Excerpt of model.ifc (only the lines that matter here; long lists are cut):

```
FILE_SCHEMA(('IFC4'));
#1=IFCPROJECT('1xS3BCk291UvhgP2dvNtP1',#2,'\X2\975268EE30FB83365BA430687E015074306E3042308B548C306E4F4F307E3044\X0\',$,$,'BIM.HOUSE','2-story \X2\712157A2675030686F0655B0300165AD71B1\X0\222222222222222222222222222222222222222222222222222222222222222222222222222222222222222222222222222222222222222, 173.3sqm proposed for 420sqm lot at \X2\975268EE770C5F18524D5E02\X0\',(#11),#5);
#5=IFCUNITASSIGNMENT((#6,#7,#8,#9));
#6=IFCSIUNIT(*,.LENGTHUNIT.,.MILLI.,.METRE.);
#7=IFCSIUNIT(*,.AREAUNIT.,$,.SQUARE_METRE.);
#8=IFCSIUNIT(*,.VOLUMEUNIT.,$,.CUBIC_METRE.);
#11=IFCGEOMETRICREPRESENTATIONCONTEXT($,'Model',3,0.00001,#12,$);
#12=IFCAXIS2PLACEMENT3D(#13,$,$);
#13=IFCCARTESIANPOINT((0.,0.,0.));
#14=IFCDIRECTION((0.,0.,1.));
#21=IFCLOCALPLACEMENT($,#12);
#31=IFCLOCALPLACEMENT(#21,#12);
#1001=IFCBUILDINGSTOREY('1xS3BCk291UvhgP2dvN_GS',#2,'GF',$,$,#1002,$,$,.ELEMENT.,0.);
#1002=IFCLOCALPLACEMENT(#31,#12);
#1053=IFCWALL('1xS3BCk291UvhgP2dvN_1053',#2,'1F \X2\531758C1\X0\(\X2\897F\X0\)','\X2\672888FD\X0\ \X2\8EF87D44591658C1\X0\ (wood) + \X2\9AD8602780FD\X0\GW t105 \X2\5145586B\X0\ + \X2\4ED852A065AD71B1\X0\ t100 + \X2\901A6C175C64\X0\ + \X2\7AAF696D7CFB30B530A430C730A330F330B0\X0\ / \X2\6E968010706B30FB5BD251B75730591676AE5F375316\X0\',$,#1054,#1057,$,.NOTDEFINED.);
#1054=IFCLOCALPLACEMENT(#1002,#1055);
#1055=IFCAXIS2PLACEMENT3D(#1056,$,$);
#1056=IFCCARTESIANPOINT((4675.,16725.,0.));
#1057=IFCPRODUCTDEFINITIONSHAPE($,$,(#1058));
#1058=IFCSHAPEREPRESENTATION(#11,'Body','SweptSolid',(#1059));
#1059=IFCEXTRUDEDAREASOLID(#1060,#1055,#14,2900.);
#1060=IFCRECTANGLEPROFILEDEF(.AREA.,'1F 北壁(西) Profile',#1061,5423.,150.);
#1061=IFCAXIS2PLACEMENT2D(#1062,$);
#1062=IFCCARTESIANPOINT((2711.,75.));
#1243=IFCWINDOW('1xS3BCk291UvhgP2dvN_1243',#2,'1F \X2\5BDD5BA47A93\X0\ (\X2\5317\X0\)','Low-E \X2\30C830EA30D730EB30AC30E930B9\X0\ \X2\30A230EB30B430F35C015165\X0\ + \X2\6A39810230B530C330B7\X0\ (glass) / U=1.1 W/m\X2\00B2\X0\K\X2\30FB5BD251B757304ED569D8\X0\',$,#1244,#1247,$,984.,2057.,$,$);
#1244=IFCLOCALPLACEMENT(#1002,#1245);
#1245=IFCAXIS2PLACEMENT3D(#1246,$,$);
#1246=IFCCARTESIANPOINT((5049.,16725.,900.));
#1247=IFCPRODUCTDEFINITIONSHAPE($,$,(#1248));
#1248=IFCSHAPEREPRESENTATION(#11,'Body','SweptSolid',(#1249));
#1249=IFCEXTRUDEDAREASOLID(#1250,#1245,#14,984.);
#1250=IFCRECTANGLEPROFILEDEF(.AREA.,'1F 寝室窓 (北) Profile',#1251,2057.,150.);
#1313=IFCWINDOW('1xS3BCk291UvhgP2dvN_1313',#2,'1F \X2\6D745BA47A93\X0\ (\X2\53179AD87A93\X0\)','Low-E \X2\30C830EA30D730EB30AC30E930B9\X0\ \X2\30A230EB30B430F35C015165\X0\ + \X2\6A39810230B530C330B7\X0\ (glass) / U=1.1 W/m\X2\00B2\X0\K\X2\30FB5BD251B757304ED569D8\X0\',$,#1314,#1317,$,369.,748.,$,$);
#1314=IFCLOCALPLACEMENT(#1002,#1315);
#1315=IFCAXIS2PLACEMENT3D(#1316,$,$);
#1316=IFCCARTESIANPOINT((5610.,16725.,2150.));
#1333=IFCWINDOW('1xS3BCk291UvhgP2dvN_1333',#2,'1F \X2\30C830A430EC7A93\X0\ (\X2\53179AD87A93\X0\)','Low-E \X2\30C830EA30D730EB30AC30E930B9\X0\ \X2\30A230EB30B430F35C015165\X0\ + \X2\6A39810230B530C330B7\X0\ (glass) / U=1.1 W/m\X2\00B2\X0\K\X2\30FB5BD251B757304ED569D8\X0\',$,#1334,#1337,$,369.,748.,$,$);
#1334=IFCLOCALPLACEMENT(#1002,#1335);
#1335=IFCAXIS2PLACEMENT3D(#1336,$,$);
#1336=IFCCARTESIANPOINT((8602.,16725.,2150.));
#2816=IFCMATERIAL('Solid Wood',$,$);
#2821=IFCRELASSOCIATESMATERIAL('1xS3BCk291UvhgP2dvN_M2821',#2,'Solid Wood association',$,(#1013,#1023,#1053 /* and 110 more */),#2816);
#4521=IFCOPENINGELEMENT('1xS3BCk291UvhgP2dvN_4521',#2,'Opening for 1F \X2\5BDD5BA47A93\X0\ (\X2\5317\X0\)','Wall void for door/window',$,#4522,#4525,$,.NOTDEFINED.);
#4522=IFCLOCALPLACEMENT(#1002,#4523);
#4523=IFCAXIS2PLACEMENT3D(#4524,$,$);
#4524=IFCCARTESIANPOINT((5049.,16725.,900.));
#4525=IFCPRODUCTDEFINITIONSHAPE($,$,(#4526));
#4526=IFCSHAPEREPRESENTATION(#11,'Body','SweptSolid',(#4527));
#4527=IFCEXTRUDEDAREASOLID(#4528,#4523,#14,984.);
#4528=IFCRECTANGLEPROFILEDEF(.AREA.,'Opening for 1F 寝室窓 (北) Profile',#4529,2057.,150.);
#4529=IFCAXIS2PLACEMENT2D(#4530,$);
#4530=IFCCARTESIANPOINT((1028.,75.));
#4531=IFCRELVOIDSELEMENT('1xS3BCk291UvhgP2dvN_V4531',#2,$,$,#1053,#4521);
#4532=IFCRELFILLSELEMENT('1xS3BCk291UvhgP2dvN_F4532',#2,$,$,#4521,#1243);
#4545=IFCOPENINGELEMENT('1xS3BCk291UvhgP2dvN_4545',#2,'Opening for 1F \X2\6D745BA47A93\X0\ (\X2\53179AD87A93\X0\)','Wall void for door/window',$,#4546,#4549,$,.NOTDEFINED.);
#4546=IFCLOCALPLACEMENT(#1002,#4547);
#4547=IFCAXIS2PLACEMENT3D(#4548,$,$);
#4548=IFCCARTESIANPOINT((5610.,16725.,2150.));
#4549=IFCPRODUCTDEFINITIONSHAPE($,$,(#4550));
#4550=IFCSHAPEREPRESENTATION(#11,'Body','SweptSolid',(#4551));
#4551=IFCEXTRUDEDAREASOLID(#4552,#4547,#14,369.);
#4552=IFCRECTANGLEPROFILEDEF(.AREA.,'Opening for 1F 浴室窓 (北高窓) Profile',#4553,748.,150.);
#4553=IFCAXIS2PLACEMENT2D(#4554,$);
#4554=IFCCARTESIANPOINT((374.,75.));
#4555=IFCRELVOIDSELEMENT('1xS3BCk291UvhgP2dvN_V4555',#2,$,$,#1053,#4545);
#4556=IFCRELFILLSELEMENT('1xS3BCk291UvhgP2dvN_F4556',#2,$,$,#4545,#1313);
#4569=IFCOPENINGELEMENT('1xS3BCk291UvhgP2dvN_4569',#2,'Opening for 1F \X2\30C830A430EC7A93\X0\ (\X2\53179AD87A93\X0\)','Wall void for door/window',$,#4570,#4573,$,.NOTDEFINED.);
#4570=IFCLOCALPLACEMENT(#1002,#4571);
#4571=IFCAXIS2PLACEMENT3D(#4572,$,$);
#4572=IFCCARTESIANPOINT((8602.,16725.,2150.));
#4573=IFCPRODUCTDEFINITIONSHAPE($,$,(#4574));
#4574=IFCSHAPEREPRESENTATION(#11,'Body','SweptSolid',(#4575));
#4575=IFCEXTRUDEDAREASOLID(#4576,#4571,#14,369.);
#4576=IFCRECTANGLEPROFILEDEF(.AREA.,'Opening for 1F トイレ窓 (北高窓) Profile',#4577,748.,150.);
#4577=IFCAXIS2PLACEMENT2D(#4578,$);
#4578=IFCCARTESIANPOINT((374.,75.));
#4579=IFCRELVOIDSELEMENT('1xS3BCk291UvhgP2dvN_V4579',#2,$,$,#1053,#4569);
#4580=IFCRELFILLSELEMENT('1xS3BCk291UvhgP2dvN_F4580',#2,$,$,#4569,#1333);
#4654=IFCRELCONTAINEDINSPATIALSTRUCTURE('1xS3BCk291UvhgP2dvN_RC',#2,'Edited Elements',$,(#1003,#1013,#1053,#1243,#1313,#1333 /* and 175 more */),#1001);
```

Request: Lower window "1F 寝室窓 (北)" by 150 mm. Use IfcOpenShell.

```python
import numpy as np
import ifcopenshell
import ifcopenshell.api.geometry
import ifcopenshell.util.placement
import ifcopenshell.util.unit

model = ifcopenshell.open("model.ifc")
unit_scale = ifcopenshell.util.unit.calculate_unit_scale(model)

window = model.by_guid("1xS3BCk291UvhgP2dvN_1243")
opening = window.FillsVoids[0].RelatingOpeningElement
dz = -150.0

shift = np.array([0.0, 0.0, dz])
# The window is not placed relative to its opening, so move both.
for product in (opening, window):
    matrix = ifcopenshell.util.placement.get_local_placement(product.ObjectPlacement)
    matrix[:3, 3] += shift
    ifcopenshell.api.geometry.edit_object_placement(model, product=product, matrix=matrix, is_si=False)

print(f"moved by {dz * unit_scale:+.3f} m")

model.write("model-out.ifc")
```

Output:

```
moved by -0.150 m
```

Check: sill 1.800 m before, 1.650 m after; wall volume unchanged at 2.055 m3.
